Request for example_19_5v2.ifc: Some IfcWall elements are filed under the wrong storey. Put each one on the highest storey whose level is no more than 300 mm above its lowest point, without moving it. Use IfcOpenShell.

First a look at what the model holds.

```python
import ifcopenshell
import ifcopenshell.util.element
import ifcopenshell.util.placement

model = ifcopenshell.open("example_19_5v2.ifc")
print(model.schema)
for storey in model.by_type("IfcBuildingStorey"):
    level = ifcopenshell.util.placement.get_storey_elevation(storey)
    count = sum(e.is_a("IfcWall") for e in ifcopenshell.util.element.get_contained(storey))
    print(storey.id(), storey.Name, round(level, 3), count, sep=" | ")
```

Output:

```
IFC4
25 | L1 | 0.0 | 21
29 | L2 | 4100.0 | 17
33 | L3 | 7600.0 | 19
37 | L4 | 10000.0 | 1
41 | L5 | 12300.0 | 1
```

```python
import ifcopenshell
import ifcopenshell.api.spatial
import ifcopenshell.geom
import ifcopenshell.util.element
import ifcopenshell.util.placement
import ifcopenshell.util.shape
import ifcopenshell.util.unit

model = ifcopenshell.open("example_19_5v2.ifc")
unit_scale = ifcopenshell.util.unit.calculate_unit_scale(model)
settings = ifcopenshell.geom.settings()

levels = sorted(
    ((ifcopenshell.util.placement.get_storey_elevation(s) * unit_scale, s) for s in model.by_type("IfcBuildingStorey")),
    key=lambda pair: pair[0],
)

for e in model.by_type("IfcWall"):
    current = e.ContainedInStructure[0].RelatingStructure if e.ContainedInStructure else None
    if current is None or not current.is_a("IfcBuildingStorey"):
        continue
    shape = ifcopenshell.geom.create_shape(settings, e)
    bottom = ifcopenshell.util.shape.get_shape_bottom_elevation(shape, shape.geometry)
    below = [s for level, s in levels if level <= bottom + 0.3]
    storey = below[-1] if below else levels[0][1]
    if storey != current:
        # assign_container keeps the world position.
        ifcopenshell.api.spatial.assign_container(model, products=[e], relating_structure=storey)
        print(e.id(), current.Name, "->", storey.Name)

model.write("example_19_5v2_rev.ifc")
```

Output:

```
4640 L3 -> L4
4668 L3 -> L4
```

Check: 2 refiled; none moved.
